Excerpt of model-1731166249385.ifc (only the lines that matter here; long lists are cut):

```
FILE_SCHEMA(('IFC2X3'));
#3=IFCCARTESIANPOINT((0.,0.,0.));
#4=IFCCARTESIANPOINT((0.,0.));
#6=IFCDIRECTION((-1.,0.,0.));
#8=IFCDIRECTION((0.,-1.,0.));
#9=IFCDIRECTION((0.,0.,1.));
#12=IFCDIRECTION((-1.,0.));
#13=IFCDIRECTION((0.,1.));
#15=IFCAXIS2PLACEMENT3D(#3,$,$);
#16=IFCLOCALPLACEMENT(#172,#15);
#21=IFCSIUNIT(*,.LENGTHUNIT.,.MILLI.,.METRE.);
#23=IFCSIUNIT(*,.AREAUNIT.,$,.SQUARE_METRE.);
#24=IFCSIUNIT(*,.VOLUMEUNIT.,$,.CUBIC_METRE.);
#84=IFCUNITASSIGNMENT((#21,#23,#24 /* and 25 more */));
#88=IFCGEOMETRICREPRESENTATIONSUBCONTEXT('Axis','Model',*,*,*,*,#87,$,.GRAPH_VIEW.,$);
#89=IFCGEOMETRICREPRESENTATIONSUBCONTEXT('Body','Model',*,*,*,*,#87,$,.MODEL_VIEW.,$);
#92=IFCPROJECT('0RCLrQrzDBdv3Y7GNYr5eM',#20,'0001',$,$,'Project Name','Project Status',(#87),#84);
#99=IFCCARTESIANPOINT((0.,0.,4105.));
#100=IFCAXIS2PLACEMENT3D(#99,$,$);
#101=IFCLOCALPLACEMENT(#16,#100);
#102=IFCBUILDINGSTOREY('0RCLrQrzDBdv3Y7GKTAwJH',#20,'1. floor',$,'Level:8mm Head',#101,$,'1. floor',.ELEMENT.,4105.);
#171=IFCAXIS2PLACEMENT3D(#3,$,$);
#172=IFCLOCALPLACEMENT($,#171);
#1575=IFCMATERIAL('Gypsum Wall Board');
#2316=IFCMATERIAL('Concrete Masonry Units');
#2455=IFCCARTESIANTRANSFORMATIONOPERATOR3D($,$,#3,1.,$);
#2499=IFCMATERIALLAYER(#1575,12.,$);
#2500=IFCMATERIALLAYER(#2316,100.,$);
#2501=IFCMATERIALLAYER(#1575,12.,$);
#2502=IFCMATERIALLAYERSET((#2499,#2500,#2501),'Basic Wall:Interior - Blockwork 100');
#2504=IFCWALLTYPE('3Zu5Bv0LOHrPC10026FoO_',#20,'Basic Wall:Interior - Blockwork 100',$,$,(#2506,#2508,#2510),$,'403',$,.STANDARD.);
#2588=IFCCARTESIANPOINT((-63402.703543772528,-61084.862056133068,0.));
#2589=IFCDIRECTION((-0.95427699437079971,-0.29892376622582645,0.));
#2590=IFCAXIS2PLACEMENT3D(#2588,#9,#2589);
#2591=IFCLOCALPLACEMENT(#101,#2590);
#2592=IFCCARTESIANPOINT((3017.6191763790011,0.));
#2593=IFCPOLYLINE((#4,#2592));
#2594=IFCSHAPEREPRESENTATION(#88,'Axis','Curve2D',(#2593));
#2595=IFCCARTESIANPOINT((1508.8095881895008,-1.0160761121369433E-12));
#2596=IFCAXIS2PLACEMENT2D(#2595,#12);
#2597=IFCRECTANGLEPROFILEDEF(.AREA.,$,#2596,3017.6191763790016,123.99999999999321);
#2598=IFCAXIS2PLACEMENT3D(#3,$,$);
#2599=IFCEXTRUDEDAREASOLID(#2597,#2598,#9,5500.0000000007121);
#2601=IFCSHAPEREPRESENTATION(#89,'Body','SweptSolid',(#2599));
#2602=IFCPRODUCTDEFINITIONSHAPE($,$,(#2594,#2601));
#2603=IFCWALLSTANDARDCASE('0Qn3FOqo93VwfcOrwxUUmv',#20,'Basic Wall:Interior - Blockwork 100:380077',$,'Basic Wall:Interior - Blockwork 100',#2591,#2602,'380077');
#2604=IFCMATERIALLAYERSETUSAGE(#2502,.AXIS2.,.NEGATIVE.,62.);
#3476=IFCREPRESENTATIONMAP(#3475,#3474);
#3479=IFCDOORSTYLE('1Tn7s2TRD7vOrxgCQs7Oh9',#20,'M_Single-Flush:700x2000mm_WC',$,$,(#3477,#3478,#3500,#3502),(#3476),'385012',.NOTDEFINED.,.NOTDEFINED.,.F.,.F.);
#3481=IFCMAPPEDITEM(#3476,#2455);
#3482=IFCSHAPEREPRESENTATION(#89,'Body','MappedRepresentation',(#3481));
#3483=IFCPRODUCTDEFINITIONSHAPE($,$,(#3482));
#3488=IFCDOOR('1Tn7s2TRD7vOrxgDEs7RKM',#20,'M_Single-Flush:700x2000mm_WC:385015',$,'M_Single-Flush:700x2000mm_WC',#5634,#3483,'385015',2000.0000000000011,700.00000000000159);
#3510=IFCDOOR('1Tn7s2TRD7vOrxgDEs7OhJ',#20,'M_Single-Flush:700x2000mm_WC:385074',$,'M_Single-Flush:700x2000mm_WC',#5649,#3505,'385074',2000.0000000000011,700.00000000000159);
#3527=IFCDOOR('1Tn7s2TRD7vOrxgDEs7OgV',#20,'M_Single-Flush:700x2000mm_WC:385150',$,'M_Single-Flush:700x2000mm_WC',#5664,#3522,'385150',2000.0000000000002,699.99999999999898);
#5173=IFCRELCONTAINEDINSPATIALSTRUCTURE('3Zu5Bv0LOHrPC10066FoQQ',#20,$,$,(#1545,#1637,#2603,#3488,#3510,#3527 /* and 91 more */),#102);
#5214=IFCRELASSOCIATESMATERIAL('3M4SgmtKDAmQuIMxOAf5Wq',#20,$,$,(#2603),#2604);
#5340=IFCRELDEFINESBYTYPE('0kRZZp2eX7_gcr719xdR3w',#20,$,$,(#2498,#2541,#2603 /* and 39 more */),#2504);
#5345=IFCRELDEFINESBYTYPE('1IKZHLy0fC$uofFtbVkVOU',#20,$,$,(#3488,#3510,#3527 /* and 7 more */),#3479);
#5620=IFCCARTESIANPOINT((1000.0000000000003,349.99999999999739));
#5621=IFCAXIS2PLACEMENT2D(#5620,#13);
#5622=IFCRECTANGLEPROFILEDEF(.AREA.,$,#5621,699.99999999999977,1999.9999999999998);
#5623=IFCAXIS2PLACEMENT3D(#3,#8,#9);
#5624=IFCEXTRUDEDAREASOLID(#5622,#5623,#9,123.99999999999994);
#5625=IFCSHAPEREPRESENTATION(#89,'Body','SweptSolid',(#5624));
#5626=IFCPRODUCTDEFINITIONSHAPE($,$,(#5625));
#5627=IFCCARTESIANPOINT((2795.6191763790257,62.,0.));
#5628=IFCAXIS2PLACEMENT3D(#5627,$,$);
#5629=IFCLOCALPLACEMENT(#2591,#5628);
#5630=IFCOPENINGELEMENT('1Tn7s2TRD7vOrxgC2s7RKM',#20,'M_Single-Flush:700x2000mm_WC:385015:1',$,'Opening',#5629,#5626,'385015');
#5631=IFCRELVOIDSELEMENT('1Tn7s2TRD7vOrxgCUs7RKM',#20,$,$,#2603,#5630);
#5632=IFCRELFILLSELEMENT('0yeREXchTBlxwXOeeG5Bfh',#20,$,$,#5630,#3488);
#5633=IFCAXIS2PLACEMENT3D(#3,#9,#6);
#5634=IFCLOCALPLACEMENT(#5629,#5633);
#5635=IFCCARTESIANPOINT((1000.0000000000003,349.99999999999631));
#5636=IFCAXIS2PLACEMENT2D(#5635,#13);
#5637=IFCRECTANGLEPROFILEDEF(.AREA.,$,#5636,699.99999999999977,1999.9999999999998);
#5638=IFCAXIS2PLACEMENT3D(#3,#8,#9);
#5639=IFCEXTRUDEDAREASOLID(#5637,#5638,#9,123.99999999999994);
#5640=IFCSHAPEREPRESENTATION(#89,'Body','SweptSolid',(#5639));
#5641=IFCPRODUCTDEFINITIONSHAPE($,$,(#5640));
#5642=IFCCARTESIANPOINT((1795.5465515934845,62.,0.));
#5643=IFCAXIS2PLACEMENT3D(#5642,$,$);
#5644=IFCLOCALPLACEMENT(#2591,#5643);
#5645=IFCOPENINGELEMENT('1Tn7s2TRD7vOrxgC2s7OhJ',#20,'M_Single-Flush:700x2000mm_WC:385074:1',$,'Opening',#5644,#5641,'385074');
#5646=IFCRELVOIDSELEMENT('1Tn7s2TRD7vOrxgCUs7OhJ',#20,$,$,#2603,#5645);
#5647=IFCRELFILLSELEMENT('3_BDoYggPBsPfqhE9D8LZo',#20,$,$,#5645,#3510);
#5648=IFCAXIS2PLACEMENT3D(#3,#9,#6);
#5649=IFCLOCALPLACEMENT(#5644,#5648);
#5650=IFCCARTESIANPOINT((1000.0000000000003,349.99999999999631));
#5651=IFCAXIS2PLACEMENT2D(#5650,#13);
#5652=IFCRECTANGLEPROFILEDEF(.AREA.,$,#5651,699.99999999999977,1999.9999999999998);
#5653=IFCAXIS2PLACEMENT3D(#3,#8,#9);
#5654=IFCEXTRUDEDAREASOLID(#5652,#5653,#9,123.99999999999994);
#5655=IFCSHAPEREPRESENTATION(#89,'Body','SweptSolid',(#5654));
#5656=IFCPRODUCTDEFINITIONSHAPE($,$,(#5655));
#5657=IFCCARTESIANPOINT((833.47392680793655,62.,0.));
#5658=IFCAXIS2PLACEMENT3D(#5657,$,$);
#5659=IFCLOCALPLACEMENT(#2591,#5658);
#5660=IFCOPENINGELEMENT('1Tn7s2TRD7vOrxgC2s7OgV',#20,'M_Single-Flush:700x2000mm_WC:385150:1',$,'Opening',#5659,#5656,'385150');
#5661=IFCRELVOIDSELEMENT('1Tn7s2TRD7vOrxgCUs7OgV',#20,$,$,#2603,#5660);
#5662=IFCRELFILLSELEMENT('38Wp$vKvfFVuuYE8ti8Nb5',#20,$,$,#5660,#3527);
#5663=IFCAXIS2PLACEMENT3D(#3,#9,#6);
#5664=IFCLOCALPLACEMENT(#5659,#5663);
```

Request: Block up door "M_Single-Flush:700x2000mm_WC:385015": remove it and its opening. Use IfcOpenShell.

```python
import ifcopenshell
import ifcopenshell.api.feature
import ifcopenshell.api.root
import ifcopenshell.geom
import ifcopenshell.util.shape

model = ifcopenshell.open("model-1731166249385.ifc")
settings = ifcopenshell.geom.settings()


def volume(element):
    """Net volume in cubic metres, openings subtracted."""
    shape = ifcopenshell.geom.create_shape(settings, element)
    return ifcopenshell.util.shape.get_volume(shape.geometry)


door = model.by_guid("1Tn7s2TRD7vOrxgDEs7RKM")
opening = door.FillsVoids[0].RelatingOpeningElement
wall = opening.VoidsElements[0].RelatingBuildingElement
before = volume(wall)

ifcopenshell.api.root.remove_product(model, product=door)
ifcopenshell.api.feature.remove_feature(model, feature=opening)

after = volume(wall)

print(f"wall volume {before:.3f} -> {after:.3f} m3")

model.write("model-1731166249385_v2.ifc")
```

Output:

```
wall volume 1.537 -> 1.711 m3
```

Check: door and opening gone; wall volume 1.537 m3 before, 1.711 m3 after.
